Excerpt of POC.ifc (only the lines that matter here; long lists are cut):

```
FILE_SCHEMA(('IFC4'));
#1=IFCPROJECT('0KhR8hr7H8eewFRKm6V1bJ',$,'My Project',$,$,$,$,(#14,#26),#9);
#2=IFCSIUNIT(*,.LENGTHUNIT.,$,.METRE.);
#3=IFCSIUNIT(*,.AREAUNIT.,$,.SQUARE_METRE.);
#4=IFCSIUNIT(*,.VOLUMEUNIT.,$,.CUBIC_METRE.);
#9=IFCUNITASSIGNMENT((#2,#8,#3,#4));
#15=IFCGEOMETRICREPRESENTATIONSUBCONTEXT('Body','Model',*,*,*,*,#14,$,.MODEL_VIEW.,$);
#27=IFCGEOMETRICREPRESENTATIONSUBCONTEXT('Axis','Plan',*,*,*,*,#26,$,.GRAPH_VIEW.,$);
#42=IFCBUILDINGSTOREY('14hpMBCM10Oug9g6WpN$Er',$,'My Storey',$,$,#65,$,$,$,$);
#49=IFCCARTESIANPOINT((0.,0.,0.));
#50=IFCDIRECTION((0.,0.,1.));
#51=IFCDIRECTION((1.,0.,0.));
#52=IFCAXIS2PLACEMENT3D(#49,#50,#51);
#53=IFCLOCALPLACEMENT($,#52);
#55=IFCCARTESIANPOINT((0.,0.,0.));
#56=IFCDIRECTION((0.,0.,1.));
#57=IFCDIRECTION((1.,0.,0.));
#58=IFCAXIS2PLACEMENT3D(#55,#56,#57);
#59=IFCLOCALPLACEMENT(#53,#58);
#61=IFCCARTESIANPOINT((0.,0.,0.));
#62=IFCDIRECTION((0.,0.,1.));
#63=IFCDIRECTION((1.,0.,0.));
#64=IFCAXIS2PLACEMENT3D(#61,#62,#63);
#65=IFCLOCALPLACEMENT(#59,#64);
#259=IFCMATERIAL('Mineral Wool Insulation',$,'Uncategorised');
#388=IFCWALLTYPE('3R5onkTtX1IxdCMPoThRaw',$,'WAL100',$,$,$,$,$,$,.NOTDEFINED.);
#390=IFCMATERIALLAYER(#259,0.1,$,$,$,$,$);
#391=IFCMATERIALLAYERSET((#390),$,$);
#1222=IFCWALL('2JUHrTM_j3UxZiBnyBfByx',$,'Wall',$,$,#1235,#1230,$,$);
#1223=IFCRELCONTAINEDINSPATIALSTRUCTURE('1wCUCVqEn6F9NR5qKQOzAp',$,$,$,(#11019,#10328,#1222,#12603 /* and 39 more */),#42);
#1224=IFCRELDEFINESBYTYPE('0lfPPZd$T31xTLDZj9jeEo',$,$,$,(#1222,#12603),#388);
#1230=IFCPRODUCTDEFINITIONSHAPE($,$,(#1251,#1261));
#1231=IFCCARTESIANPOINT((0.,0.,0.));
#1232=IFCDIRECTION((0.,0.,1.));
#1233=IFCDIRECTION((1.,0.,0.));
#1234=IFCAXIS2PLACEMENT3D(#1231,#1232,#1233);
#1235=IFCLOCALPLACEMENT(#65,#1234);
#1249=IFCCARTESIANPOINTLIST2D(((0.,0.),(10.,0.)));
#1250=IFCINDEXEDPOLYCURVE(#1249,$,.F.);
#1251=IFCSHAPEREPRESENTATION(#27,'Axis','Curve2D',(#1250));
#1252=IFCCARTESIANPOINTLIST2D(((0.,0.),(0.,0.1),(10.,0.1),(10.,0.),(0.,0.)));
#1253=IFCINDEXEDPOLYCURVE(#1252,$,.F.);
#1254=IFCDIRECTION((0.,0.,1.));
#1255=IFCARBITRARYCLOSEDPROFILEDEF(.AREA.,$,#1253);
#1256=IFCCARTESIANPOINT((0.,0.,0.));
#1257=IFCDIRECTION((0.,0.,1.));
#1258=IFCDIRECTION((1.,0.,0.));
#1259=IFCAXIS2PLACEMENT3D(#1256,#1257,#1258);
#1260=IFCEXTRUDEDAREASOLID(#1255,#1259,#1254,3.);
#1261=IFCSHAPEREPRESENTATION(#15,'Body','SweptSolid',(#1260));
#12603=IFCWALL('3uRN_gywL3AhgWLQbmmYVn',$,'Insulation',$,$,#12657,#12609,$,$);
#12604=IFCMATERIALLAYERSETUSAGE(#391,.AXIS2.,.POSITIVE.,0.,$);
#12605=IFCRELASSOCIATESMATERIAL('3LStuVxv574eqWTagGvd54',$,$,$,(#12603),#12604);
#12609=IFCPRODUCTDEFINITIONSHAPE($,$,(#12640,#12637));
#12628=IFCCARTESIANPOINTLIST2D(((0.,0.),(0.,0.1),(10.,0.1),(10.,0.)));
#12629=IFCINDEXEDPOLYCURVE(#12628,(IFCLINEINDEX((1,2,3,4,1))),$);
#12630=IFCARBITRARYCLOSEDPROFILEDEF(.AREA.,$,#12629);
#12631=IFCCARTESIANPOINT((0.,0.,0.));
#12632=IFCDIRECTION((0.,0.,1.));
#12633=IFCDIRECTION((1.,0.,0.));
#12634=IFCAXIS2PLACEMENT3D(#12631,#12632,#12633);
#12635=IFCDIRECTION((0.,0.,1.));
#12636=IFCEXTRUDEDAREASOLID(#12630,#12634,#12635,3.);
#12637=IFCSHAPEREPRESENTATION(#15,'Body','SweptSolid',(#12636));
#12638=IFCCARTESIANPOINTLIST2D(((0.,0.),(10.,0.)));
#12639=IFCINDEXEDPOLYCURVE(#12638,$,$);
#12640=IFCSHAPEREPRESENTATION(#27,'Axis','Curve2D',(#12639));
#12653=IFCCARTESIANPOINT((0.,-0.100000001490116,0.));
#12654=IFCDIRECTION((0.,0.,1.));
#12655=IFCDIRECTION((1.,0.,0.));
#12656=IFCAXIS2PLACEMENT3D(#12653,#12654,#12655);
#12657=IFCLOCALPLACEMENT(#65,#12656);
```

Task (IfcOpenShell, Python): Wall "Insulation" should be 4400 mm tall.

```python
import ifcopenshell
import ifcopenshell.geom
import ifcopenshell.util.representation
import ifcopenshell.util.shape
import ifcopenshell.util.unit

model = ifcopenshell.open("POC.ifc")
unit_scale = ifcopenshell.util.unit.calculate_unit_scale(model)
settings = ifcopenshell.geom.settings()


def volume(element):
    """Net volume in cubic metres, openings subtracted."""
    shape = ifcopenshell.geom.create_shape(settings, element)
    return ifcopenshell.util.shape.get_volume(shape.geometry)


wall = model.by_guid("3uRN_gywL3AhgWLQbmmYVn")
before = volume(wall)

body = ifcopenshell.util.representation.get_representation(wall, "Model", "Body")
solid = body.Items[0]
old_height = solid.Depth
solid.Depth = 4.4 / unit_scale
after = volume(wall)

print(f"height {old_height:g} -> {solid.Depth:g}, volume {before:.3f} -> {after:.3f} m3")

model.write("POC_updated.ifc")
```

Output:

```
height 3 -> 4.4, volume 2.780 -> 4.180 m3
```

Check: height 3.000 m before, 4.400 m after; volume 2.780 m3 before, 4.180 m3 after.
